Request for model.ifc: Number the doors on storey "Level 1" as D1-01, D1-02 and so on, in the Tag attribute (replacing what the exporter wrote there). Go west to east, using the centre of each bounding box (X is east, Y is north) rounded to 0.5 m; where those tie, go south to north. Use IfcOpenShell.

First a look at what the model holds.

```python
import ifcopenshell
import ifcopenshell.util.element
import ifcopenshell.util.placement

model = ifcopenshell.open("model.ifc")
print(model.schema)
storey = next(s for s in model.by_type("IfcBuildingStorey") if s.Name == "Level 1")
doors = [e for e in ifcopenshell.util.element.get_decomposition(storey) if e.is_a("IfcDoor")]
for e in sorted(doors, key=lambda e: e.id()):
    origin = ifcopenshell.util.placement.get_local_placement(e.ObjectPlacement)[:3, 3]
    print(e.id(), e.Tag, e.Name, origin.round(2) + 0.0, sep=" | ")
```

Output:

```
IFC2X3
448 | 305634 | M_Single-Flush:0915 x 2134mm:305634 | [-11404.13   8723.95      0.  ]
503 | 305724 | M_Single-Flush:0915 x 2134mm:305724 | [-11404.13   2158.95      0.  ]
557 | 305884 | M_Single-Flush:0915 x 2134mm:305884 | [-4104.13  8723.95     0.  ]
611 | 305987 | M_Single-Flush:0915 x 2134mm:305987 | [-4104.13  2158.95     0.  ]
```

```python
import ifcopenshell
import ifcopenshell.geom
import ifcopenshell.util.element
import ifcopenshell.util.shape

model = ifcopenshell.open("model.ifc")
settings = ifcopenshell.geom.settings()
settings.set("use-world-coords", True)


def centre(element):
    shape = ifcopenshell.geom.create_shape(settings, element)
    return ifcopenshell.util.shape.get_bbox_centroid(shape.geometry)


storey = next(s for s in model.by_type("IfcBuildingStorey") if s.Name == "Level 1")
doors = [e for e in ifcopenshell.util.element.get_decomposition(storey) if e.is_a("IfcDoor")]

# Insertion points can sit at a corner or the storey origin, so sort by the geometry (in metres).
centres = {e: centre(e) for e in doors}
doors.sort(key=lambda e: (round(centres[e][0] / 0.5), centres[e][1]))

for i, e in enumerate(doors, start=1):
    number = f"D1-{i:02d}"
    e.Tag = number
    print(e.id(), number)

model.write("model_rev.ifc")
```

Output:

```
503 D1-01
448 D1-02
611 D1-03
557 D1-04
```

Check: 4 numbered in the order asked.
